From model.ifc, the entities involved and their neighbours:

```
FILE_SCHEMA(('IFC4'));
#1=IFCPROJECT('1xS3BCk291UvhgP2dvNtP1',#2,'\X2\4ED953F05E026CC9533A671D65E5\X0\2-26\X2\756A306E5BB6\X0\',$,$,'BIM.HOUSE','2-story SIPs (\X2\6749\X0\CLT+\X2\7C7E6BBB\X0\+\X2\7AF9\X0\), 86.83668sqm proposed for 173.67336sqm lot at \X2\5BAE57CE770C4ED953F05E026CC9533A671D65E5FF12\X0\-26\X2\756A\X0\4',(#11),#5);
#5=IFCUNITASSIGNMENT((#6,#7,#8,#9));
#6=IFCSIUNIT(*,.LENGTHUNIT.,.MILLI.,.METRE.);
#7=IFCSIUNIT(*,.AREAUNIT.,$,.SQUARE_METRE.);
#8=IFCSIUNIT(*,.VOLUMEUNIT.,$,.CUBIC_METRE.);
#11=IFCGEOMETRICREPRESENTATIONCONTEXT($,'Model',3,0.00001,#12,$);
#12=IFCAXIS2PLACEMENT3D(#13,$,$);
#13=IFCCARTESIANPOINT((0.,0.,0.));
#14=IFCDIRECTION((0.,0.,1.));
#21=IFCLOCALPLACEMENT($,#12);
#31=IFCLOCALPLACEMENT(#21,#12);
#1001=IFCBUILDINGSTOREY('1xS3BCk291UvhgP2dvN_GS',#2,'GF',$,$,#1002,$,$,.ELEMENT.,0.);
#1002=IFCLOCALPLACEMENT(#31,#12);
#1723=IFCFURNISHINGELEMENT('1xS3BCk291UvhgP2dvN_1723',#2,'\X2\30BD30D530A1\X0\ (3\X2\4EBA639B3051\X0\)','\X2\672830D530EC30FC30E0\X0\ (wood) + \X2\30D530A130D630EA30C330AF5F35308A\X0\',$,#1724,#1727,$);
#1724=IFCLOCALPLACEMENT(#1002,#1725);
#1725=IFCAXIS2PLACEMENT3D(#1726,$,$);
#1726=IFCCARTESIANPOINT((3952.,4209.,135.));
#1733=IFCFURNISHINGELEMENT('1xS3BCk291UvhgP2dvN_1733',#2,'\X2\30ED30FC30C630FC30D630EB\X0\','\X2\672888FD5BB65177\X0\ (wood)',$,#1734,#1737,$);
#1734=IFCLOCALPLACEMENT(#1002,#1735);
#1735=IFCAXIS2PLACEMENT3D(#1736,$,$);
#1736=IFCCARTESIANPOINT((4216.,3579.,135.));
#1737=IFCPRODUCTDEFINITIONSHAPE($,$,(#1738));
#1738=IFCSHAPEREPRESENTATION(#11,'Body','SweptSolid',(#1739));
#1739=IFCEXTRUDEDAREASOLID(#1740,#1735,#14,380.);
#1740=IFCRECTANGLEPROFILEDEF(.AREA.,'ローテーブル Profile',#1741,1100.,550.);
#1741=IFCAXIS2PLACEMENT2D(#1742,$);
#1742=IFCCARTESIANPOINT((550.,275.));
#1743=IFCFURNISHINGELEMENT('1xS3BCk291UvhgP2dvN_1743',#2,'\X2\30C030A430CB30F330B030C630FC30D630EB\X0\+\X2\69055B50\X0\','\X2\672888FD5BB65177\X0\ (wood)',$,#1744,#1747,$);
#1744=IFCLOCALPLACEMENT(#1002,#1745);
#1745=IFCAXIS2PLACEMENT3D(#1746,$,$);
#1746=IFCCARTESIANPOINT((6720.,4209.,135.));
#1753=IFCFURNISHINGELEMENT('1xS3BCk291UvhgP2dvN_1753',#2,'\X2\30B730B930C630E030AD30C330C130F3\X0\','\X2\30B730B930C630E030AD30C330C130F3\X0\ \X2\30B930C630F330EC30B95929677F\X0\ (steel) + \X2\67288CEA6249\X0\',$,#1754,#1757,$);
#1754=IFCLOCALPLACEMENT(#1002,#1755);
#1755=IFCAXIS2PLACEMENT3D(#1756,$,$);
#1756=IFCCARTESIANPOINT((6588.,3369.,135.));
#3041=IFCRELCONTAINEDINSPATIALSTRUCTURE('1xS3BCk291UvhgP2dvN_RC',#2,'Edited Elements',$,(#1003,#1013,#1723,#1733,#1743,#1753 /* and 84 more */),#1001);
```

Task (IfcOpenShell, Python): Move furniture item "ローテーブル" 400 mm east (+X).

```python
import ifcopenshell
import ifcopenshell.api.geometry
import ifcopenshell.util.placement
import ifcopenshell.util.unit

model = ifcopenshell.open("model.ifc")
unit_scale = ifcopenshell.util.unit.calculate_unit_scale(model)

item = model.by_guid("1xS3BCk291UvhgP2dvN_1733")
matrix = ifcopenshell.util.placement.get_local_placement(item.ObjectPlacement)
matrix[0, 3] += 0.4 / unit_scale
ifcopenshell.api.geometry.edit_object_placement(model, product=item, matrix=matrix, is_si=False)

print(ifcopenshell.util.placement.get_local_placement(item.ObjectPlacement).round(3) + 0.0)

model.write("model-out.ifc")
```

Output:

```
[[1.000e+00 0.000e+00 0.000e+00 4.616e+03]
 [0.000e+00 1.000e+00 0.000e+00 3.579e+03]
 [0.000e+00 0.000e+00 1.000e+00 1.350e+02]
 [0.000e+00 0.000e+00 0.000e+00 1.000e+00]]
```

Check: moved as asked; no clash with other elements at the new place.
